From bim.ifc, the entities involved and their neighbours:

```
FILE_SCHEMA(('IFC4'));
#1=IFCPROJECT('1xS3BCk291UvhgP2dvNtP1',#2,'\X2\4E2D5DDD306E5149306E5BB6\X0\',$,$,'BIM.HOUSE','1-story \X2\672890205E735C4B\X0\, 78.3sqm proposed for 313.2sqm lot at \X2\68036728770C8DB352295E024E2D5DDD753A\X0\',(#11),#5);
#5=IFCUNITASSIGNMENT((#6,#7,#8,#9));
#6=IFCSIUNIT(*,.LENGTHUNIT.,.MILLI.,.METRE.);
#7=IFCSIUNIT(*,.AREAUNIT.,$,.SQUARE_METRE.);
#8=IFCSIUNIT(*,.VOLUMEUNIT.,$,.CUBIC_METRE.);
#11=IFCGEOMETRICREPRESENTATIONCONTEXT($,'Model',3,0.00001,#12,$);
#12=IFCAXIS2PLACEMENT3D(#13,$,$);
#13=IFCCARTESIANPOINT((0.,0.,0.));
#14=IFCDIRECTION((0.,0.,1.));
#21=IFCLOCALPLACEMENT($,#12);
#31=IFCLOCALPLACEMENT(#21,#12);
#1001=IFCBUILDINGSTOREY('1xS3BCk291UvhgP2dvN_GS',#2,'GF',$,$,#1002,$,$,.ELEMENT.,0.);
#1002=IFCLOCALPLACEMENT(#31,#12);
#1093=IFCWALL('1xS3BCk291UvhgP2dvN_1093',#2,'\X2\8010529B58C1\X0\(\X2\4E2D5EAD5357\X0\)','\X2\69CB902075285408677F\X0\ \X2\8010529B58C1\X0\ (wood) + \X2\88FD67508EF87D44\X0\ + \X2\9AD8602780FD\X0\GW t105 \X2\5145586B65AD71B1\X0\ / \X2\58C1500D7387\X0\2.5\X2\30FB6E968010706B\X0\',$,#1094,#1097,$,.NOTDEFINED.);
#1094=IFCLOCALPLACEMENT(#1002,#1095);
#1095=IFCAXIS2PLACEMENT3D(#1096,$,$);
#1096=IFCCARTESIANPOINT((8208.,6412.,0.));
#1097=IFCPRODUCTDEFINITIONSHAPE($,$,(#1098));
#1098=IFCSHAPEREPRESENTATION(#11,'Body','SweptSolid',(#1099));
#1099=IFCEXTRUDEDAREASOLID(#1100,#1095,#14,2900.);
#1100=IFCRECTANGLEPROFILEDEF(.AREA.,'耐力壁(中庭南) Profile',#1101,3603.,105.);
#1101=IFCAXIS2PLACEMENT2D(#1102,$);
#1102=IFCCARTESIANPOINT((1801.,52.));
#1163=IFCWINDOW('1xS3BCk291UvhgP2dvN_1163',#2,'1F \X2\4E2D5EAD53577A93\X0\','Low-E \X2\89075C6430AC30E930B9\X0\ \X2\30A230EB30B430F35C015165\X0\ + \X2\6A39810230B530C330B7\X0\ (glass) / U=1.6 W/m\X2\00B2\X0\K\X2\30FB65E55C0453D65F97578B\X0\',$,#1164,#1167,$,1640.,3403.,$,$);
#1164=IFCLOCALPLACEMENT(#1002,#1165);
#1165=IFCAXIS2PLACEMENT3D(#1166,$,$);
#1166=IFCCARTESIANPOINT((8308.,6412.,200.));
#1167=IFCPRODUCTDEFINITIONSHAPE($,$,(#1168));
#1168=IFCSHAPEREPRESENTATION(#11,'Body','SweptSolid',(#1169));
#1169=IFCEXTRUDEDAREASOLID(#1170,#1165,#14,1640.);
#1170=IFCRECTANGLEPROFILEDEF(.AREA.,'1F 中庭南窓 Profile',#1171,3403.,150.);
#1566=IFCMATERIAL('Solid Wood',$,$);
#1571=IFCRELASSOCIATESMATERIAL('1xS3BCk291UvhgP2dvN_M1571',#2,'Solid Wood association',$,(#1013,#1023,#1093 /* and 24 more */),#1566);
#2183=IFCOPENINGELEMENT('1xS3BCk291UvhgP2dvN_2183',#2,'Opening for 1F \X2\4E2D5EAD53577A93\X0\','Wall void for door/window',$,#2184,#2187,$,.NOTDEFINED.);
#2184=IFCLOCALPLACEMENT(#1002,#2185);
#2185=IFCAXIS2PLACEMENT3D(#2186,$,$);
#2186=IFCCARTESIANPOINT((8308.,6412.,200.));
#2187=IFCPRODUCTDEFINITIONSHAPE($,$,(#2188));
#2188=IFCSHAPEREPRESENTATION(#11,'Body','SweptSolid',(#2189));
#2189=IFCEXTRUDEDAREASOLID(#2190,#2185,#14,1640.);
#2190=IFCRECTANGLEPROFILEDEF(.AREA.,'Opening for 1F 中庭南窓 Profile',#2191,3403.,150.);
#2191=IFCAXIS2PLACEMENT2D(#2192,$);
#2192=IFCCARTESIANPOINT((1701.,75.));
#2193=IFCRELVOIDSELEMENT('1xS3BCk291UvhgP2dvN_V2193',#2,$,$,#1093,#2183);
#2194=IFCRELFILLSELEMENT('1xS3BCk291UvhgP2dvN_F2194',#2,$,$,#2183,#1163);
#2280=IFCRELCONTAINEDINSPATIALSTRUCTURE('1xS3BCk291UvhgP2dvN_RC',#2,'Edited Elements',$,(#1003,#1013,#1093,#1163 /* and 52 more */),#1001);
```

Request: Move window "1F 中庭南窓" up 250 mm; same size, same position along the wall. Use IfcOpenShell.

```python
import numpy as np
import ifcopenshell
import ifcopenshell.api.geometry
import ifcopenshell.util.placement
import ifcopenshell.util.unit

model = ifcopenshell.open("bim.ifc")
unit_scale = ifcopenshell.util.unit.calculate_unit_scale(model)

window = model.by_guid("1xS3BCk291UvhgP2dvN_1163")
opening = window.FillsVoids[0].RelatingOpeningElement
dz = 0.25 / unit_scale

shift = np.array([0.0, 0.0, dz])
# The window is not placed relative to its opening, so move both.
for product in (opening, window):
    matrix = ifcopenshell.util.placement.get_local_placement(product.ObjectPlacement)
    matrix[:3, 3] += shift
    ifcopenshell.api.geometry.edit_object_placement(model, product=product, matrix=matrix, is_si=False)

print(f"moved by {dz * unit_scale:+.3f} m")

model.write("bim_updated.ifc")
```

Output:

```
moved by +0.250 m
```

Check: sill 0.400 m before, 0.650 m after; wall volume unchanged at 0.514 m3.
